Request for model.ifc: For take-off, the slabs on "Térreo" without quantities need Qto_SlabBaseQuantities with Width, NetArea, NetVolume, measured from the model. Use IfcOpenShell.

First a look at what the model holds.

```python
import ifcopenshell
import ifcopenshell.util.element
import ifcopenshell.util.unit

model = ifcopenshell.open("model.ifc")
print(model.schema)
for unit_type in ("LENGTHUNIT", "AREAUNIT", "VOLUMEUNIT"):
    print(unit_type, ifcopenshell.util.unit.calculate_unit_scale(model, unit_type))
storey = next(s for s in model.by_type("IfcBuildingStorey") if s.Name == "Térreo")
slabs = [e for e in ifcopenshell.util.element.get_decomposition(storey) if e.is_a("IfcSlab")]
for e in sorted(slabs, key=lambda e: e.id()):
    print(e.id(), e.is_a(), e.Name, list(ifcopenshell.util.element.get_psets(e, qtos_only=True)), sep=" | ")
```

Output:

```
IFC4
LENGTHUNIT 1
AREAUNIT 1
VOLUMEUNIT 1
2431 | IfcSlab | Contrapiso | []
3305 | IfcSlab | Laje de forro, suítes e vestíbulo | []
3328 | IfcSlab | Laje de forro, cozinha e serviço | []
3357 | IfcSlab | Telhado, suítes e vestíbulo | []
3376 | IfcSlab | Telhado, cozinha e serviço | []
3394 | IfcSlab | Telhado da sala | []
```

```python
import ifcopenshell
import ifcopenshell.api.pset
import ifcopenshell.geom
import ifcopenshell.util.element
import ifcopenshell.util.shape
import ifcopenshell.util.unit

model = ifcopenshell.open("model.ifc")
unit_scale = ifcopenshell.util.unit.calculate_unit_scale(model)
area_scale = ifcopenshell.util.unit.calculate_unit_scale(model, "AREAUNIT")
volume_scale = ifcopenshell.util.unit.calculate_unit_scale(model, "VOLUMEUNIT")
settings = ifcopenshell.geom.settings()

storey = next(s for s in model.by_type("IfcBuildingStorey") if s.Name == "Térreo")
slabs = [e for e in ifcopenshell.util.element.get_decomposition(storey) if e.is_a("IfcSlab")]

for e in sorted(slabs, key=lambda e: e.id()):
    if ifcopenshell.util.element.get_psets(e, qtos_only=True, should_inherit=False):
        continue
    # Geometry comes back in metres, in the element's own axes.
    shape = ifcopenshell.geom.create_shape(settings, e)
    values = {
        "Width": ifcopenshell.util.shape.get_z(shape.geometry) / unit_scale,
        "NetArea": ifcopenshell.util.shape.get_footprint_area(shape.geometry) / area_scale,
        "NetVolume": ifcopenshell.util.shape.get_volume(shape.geometry) / volume_scale,
    }
    qto = ifcopenshell.api.pset.add_qto(model, product=e, name="Qto_SlabBaseQuantities")
    ifcopenshell.api.pset.edit_qto(model, qto=qto, properties=values)
    print(e.id(), {k: round(v, 3) for k, v in values.items()})

model.write("model_updated.ifc")
```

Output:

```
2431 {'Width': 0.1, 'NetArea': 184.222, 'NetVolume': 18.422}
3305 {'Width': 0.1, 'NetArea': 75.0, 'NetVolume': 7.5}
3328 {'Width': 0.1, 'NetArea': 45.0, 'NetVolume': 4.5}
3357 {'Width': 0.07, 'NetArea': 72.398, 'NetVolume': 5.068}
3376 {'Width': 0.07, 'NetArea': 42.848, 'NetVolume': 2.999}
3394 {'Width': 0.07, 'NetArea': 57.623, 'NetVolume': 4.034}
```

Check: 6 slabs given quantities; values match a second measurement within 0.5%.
